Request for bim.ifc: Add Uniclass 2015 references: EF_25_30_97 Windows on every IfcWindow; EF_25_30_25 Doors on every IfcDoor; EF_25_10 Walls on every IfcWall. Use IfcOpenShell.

First a look at what the model holds.

```python
import ifcopenshell

model = ifcopenshell.open("bim.ifc")
print(model.schema)
print("classifications:", [c.Name for c in model.by_type("IfcClassification")])
for ifc_class in ("IfcDoor", "IfcRoof", "IfcStair", "IfcWall", "IfcWindow"):
    print(ifc_class, len(model.by_type(ifc_class)))
```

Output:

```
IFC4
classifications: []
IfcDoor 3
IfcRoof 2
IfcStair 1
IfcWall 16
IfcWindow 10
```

```python
import ifcopenshell
import ifcopenshell.api.classification

model = ifcopenshell.open("bim.ifc")

system = ifcopenshell.api.classification.add_classification(model, classification="Uniclass 2015")

codes = {
    "IfcWindow": ("EF_25_30_97", "Windows"),
    "IfcDoor": ("EF_25_30_25", "Doors"),
    "IfcWall": ("EF_25_10", "Walls"),
}
for ifc_class, (code, name) in codes.items():
    products = model.by_type(ifc_class)
    ifcopenshell.api.classification.add_reference(
        model, products=products, classification=system, identification=code, name=name
    )
    print(code, len(products))

model.write("bim_rev.ifc")
```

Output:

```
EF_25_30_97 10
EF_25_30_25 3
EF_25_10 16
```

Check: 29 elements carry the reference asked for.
